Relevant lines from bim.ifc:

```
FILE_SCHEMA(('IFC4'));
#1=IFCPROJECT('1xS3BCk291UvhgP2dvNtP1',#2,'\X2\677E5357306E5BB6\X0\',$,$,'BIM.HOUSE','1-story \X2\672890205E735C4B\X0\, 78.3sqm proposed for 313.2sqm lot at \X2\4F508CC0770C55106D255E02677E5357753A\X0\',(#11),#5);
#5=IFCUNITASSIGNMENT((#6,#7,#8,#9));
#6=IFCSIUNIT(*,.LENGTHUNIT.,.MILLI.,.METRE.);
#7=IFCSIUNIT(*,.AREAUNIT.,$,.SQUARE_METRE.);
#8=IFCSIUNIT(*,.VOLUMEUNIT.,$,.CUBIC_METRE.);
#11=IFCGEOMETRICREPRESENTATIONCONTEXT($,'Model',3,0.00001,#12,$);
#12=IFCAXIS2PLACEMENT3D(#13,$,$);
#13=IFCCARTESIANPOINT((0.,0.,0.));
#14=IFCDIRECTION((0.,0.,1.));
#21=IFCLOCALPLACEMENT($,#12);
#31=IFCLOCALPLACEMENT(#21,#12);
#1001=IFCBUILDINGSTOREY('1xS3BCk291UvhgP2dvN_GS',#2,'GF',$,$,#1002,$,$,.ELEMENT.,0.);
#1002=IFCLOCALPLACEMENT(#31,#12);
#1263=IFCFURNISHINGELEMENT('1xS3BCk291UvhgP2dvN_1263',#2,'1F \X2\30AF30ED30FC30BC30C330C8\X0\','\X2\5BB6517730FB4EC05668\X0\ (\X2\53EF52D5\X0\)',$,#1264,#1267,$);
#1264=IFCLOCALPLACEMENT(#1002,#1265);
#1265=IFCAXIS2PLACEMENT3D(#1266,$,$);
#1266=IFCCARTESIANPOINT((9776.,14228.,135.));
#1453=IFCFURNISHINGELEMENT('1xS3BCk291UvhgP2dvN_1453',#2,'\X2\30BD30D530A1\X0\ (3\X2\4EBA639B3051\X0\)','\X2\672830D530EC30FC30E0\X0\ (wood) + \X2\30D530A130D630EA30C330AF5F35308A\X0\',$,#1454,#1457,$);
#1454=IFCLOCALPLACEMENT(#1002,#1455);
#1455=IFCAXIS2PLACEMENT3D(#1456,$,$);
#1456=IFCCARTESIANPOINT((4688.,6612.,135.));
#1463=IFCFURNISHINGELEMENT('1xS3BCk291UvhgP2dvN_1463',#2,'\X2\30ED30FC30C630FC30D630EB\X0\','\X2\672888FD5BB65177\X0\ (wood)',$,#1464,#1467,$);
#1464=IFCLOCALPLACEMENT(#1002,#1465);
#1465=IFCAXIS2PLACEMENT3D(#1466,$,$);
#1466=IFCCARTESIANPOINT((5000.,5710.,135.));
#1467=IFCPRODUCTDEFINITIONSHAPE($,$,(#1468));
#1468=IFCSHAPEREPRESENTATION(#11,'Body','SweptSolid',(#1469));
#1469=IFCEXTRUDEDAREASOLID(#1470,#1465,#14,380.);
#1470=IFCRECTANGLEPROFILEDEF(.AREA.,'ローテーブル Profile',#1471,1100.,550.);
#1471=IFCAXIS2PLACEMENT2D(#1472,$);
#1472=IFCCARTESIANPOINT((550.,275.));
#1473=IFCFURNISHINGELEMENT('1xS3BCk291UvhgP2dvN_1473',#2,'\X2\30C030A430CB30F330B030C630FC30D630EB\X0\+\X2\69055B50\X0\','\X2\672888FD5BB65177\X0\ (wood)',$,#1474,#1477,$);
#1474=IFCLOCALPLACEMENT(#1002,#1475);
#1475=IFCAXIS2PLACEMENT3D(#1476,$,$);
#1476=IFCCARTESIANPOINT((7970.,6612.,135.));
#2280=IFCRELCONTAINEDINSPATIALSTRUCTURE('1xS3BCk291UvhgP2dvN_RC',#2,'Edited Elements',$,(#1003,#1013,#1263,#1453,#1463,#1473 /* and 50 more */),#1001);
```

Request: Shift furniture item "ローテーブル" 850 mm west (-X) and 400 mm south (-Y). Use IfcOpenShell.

```python
import ifcopenshell
import ifcopenshell.api.geometry
import ifcopenshell.util.placement

model = ifcopenshell.open("bim.ifc")

item = model.by_guid("1xS3BCk291UvhgP2dvN_1463")
matrix = ifcopenshell.util.placement.get_local_placement(item.ObjectPlacement)
matrix[0, 3] -= 850.0
matrix[1, 3] -= 400.0
ifcopenshell.api.geometry.edit_object_placement(model, product=item, matrix=matrix, is_si=False)

print(ifcopenshell.util.placement.get_local_placement(item.ObjectPlacement).round(3) + 0.0)

model.write("bim-out.ifc")
```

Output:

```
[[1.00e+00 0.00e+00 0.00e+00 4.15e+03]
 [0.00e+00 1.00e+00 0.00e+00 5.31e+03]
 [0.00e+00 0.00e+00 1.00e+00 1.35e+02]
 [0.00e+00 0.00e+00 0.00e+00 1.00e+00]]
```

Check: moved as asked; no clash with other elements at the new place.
